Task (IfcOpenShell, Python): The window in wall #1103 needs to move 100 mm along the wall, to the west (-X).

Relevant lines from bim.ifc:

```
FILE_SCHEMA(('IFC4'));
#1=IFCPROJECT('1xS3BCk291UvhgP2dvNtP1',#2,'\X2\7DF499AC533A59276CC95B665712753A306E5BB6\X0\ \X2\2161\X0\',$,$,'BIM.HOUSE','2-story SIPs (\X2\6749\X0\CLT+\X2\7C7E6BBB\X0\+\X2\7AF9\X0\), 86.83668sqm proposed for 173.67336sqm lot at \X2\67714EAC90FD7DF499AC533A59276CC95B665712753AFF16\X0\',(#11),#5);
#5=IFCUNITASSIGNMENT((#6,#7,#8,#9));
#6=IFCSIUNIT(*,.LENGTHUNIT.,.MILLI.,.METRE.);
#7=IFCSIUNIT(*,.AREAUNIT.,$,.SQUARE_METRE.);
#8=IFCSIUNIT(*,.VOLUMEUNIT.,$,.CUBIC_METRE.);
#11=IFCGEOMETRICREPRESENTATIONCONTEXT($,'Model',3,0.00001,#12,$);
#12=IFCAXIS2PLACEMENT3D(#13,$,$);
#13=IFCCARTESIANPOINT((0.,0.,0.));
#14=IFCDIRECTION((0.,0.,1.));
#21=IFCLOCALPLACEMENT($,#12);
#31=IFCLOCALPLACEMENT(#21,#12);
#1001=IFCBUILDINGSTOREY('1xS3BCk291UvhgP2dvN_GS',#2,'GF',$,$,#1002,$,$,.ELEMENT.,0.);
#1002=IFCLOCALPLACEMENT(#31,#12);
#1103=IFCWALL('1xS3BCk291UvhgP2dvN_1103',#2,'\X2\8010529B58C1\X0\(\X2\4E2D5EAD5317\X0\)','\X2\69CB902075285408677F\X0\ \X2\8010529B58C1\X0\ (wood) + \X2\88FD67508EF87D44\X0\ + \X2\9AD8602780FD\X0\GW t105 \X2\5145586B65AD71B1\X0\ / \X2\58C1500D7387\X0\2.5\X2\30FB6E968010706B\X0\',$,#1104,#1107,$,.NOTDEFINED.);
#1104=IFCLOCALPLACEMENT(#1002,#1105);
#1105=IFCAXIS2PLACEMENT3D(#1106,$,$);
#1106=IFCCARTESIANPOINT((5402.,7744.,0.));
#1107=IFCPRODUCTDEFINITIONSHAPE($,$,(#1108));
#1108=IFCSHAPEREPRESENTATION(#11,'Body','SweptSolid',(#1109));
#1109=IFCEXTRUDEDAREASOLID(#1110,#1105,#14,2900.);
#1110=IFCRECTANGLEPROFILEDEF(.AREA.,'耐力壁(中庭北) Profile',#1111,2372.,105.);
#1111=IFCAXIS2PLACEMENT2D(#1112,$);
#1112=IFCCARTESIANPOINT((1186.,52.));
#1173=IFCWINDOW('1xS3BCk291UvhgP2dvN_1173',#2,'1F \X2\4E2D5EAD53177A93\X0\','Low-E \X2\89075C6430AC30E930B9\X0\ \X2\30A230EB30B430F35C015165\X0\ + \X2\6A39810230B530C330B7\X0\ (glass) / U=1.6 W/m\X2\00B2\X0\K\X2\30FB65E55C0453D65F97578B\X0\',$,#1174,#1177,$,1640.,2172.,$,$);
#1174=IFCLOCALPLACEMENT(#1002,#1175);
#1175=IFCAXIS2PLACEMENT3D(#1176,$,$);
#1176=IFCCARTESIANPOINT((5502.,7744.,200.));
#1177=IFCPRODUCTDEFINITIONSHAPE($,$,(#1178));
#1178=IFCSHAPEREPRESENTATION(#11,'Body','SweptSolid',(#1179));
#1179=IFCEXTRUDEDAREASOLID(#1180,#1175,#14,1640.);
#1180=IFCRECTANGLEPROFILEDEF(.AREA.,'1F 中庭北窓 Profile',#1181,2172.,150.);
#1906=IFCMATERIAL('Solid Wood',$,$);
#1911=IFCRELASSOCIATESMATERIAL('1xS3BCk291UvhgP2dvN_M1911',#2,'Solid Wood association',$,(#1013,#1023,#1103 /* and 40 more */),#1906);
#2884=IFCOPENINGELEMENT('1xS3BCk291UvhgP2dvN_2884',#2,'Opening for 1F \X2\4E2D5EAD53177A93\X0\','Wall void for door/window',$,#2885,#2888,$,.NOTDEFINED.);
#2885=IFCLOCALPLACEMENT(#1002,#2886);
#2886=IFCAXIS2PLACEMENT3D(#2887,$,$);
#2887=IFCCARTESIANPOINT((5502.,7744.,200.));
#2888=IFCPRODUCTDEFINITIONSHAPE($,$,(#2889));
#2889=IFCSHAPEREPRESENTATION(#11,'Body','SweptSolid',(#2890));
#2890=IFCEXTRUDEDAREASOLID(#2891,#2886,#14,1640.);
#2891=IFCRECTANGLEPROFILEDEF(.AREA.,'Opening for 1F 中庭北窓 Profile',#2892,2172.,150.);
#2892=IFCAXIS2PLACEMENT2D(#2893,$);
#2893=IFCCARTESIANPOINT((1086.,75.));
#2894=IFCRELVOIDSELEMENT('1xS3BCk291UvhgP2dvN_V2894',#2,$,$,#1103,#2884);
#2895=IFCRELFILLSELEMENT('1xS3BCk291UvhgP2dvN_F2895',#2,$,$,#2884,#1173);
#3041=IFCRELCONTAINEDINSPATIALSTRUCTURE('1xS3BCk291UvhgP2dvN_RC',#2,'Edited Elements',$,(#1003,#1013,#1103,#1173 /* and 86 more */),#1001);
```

```python
import ifcopenshell
import ifcopenshell.api.geometry
import ifcopenshell.util.placement
import ifcopenshell.util.unit

model = ifcopenshell.open("bim.ifc")
unit_scale = ifcopenshell.util.unit.calculate_unit_scale(model)

window = model.by_id(1173)
opening = window.FillsVoids[0].RelatingOpeningElement
wall = opening.VoidsElements[0].RelatingBuildingElement

wall_matrix = ifcopenshell.util.placement.get_local_placement(wall.ObjectPlacement)
shift = wall_matrix[:3, 0] * -0.1 / unit_scale
before = ifcopenshell.util.placement.get_local_placement(window.ObjectPlacement)[:3, 3].copy()

# The window is not placed relative to its opening, so move both.
for product in (opening, window):
    matrix = ifcopenshell.util.placement.get_local_placement(product.ObjectPlacement)
    matrix[:3, 3] += shift
    ifcopenshell.api.geometry.edit_object_placement(model, product=product, matrix=matrix, is_si=False)

after = ifcopenshell.util.placement.get_local_placement(window.ObjectPlacement)[:3, 3]
print("window moved by", (after - before).round(3) + 0.0)

model.write("bim_rev.ifc")
```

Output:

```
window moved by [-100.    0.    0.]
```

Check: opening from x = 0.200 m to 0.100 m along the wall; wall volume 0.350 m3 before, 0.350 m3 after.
